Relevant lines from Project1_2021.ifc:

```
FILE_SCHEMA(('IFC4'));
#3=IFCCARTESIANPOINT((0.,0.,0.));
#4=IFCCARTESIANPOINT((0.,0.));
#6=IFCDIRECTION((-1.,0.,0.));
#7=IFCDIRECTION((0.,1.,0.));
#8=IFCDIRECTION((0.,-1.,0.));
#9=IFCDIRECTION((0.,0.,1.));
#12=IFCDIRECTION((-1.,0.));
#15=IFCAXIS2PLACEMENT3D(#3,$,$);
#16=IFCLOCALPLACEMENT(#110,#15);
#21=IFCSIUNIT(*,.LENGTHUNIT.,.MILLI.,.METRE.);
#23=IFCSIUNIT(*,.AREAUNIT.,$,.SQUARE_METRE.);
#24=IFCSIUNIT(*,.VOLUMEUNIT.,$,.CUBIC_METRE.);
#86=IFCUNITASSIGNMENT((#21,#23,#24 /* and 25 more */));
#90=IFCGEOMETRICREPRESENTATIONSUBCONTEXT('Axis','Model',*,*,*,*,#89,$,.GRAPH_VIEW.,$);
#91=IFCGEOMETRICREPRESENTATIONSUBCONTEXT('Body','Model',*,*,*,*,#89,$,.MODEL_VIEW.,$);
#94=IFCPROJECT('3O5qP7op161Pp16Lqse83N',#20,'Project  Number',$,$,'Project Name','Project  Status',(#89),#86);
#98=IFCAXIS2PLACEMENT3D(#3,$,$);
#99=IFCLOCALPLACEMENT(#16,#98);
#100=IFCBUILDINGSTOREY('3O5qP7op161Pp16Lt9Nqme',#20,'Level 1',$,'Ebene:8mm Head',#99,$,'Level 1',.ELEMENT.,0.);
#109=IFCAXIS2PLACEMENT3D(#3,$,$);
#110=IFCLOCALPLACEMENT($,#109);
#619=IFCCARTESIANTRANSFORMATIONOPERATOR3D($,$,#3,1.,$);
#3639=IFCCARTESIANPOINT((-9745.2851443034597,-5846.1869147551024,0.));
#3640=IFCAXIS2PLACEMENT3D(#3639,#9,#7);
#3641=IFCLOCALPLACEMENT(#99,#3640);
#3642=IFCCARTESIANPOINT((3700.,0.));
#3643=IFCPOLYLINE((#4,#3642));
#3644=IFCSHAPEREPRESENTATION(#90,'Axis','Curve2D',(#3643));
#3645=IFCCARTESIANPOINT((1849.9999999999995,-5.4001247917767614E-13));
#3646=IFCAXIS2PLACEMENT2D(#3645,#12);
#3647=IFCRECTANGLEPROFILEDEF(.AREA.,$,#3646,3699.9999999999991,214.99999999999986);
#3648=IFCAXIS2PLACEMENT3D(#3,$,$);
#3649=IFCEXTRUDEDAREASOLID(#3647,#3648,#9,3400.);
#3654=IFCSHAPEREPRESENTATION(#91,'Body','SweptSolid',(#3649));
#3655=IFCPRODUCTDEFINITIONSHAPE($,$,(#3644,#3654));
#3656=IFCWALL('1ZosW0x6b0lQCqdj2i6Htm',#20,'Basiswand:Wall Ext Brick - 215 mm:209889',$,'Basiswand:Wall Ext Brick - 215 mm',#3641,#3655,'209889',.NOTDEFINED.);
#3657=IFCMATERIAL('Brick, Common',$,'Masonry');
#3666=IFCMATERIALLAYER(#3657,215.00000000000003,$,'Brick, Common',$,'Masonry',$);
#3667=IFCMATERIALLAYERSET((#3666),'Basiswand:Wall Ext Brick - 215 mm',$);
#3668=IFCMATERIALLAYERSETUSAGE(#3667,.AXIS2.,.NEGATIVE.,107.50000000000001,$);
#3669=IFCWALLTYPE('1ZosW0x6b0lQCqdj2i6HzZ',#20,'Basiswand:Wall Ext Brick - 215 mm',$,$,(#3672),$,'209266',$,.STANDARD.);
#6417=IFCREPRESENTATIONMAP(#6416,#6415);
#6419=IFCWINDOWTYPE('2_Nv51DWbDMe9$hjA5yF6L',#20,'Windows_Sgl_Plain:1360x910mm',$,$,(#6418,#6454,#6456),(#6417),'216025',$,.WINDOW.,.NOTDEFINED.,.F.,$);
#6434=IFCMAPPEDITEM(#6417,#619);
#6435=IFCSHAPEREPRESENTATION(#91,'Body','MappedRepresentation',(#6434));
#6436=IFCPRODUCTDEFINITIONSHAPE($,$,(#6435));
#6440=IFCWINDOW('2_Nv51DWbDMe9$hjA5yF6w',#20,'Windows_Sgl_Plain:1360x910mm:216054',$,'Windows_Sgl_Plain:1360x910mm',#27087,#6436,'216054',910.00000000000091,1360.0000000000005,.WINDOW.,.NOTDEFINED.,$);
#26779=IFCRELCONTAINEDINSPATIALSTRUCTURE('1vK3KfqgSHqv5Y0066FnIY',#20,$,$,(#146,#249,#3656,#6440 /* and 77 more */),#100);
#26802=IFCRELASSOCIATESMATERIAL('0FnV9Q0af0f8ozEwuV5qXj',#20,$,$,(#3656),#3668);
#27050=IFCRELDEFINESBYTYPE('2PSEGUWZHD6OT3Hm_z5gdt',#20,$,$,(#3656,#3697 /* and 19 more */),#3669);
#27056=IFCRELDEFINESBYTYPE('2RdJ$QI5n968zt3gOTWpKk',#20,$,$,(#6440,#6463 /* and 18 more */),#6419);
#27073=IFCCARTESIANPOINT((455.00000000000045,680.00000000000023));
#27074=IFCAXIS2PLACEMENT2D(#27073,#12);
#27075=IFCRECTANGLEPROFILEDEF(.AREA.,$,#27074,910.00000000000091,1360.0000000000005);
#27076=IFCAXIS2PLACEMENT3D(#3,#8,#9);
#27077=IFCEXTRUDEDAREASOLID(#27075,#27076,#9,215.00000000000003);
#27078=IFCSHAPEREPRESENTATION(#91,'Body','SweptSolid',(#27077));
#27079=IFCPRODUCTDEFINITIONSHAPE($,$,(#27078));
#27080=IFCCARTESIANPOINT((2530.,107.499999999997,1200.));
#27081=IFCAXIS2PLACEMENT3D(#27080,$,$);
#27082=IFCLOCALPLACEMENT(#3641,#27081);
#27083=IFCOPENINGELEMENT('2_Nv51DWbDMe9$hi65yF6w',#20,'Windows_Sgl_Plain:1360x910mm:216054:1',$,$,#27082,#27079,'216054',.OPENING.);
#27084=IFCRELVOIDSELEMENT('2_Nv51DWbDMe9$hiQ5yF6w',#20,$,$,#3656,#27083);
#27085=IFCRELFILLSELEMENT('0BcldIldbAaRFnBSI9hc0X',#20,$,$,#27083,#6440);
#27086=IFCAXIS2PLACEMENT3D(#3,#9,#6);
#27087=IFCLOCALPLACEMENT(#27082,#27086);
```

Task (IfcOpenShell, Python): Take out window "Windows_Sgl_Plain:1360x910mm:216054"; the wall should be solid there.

```python
import ifcopenshell
import ifcopenshell.api.feature
import ifcopenshell.api.root
import ifcopenshell.geom
import ifcopenshell.util.shape

model = ifcopenshell.open("Project1_2021.ifc")
settings = ifcopenshell.geom.settings()


def volume(element):
    """Net volume in cubic metres, openings subtracted."""
    shape = ifcopenshell.geom.create_shape(settings, element)
    return ifcopenshell.util.shape.get_volume(shape.geometry)


window = model.by_id(6440)
opening = window.FillsVoids[0].RelatingOpeningElement
wall = opening.VoidsElements[0].RelatingBuildingElement
before = volume(wall)

ifcopenshell.api.root.remove_product(model, product=window)
ifcopenshell.api.feature.remove_feature(model, feature=opening)

after = volume(wall)

print(f"wall volume {before:.3f} -> {after:.3f} m3")

model.write("Project1_2021_updated.ifc")
```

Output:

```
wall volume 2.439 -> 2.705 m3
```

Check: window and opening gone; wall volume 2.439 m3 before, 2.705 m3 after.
